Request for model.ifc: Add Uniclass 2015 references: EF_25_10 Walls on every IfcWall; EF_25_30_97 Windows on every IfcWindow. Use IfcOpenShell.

First a look at what the model holds.

```python
import ifcopenshell

model = ifcopenshell.open("model.ifc")
print(model.schema)
print("classifications:", [c.Name for c in model.by_type("IfcClassification")])
for ifc_class in ("IfcDoor", "IfcRoof", "IfcStair", "IfcWall", "IfcWindow"):
    print(ifc_class, len(model.by_type(ifc_class)))
```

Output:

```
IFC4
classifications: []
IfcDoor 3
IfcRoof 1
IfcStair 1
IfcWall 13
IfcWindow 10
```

```python
import ifcopenshell
import ifcopenshell.api.classification

model = ifcopenshell.open("model.ifc")

system = ifcopenshell.api.classification.add_classification(model, classification="Uniclass 2015")

codes = {
    "IfcWall": ("EF_25_10", "Walls"),
    "IfcWindow": ("EF_25_30_97", "Windows"),
}
for ifc_class, (code, name) in codes.items():
    products = model.by_type(ifc_class)
    ifcopenshell.api.classification.add_reference(
        model, products=products, classification=system, identification=code, name=name
    )
    print(code, len(products))

model.write("model_updated.ifc")
```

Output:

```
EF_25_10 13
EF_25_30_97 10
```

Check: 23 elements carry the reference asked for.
